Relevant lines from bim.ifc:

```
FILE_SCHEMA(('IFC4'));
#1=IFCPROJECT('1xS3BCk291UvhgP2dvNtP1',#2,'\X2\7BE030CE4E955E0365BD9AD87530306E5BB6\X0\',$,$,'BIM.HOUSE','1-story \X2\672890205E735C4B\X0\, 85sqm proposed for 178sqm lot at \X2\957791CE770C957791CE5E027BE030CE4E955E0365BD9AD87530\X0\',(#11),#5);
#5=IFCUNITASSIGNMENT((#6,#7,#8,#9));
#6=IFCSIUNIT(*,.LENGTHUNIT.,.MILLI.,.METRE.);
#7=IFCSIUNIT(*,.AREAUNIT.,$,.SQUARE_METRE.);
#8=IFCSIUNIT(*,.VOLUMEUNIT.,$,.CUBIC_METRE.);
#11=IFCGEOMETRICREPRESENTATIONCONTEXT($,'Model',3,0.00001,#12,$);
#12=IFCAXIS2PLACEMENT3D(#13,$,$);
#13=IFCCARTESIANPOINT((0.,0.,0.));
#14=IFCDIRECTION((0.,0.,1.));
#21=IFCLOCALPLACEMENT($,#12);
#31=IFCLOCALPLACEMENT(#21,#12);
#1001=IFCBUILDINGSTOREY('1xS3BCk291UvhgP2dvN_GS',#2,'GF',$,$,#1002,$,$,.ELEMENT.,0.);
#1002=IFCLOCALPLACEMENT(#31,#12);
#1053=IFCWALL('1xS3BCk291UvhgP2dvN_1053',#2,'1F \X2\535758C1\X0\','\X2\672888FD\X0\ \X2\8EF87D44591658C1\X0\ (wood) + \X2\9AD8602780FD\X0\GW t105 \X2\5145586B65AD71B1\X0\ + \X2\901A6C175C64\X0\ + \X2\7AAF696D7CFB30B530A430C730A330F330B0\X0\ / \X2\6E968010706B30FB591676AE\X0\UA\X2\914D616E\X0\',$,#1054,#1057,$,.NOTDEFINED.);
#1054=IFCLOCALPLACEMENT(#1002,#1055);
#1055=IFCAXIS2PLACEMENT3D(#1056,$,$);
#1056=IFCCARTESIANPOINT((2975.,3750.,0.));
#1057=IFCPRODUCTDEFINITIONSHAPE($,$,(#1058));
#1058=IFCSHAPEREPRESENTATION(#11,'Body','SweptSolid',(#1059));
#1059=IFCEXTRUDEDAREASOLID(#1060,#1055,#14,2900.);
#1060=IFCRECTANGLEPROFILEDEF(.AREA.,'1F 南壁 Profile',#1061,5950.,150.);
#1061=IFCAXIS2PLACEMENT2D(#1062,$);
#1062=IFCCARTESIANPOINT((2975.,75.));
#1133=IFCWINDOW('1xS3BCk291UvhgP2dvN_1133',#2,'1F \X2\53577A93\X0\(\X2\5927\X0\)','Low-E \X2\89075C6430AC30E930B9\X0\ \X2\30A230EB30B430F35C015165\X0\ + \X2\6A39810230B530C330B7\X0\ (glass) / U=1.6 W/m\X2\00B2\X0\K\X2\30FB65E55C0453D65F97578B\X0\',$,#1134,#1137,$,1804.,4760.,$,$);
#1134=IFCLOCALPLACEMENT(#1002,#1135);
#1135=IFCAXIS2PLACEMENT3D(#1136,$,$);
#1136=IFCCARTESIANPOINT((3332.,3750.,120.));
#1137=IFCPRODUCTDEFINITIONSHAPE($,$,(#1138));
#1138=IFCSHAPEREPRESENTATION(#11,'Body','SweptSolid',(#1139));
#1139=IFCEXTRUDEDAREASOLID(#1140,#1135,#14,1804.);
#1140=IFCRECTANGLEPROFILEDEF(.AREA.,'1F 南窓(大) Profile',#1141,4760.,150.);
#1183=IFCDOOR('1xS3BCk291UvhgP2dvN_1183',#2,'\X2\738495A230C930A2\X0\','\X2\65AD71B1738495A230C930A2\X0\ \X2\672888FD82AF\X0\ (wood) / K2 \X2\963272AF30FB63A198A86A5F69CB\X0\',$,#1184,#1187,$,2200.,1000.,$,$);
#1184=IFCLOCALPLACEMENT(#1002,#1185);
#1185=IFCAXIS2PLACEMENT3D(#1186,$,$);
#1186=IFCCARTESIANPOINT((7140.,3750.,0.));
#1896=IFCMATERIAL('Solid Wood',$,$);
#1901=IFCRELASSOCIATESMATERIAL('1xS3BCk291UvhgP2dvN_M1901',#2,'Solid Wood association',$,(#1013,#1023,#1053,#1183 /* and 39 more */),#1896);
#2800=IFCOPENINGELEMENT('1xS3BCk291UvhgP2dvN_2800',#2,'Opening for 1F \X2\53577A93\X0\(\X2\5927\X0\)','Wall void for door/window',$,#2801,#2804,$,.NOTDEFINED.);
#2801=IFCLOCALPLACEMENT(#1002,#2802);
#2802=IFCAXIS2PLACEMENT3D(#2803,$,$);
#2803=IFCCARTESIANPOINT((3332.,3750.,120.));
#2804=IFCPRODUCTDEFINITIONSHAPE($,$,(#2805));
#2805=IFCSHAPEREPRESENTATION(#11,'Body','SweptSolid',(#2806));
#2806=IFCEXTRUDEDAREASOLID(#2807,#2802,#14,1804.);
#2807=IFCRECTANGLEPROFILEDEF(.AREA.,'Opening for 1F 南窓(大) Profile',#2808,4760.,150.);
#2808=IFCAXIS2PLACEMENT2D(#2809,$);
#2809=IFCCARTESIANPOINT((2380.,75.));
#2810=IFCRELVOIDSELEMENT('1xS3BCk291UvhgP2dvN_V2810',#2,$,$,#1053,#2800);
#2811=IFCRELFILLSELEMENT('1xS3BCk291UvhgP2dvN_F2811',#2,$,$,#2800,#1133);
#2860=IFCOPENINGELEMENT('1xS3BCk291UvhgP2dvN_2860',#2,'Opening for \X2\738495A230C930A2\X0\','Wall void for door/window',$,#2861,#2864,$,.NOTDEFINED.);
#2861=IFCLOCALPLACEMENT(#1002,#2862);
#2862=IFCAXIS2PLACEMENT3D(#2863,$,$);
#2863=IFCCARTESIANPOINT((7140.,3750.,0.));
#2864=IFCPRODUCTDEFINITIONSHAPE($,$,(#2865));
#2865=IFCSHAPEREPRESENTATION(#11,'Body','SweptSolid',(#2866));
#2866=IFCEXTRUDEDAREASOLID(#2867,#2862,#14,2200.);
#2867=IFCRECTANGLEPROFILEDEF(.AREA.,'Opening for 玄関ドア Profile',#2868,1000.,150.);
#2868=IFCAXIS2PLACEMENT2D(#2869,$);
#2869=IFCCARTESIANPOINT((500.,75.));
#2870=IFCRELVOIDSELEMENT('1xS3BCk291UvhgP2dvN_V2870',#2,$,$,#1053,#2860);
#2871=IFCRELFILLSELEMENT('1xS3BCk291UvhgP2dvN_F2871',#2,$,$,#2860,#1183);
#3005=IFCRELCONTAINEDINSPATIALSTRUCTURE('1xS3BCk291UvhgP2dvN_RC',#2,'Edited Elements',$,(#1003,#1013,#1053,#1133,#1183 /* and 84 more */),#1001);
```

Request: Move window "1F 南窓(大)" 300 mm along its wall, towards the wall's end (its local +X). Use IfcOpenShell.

```python
import ifcopenshell
import ifcopenshell.api.geometry
import ifcopenshell.util.placement

model = ifcopenshell.open("bim.ifc")

window = model.by_guid("1xS3BCk291UvhgP2dvN_1133")
opening = window.FillsVoids[0].RelatingOpeningElement
wall = opening.VoidsElements[0].RelatingBuildingElement

wall_matrix = ifcopenshell.util.placement.get_local_placement(wall.ObjectPlacement)
shift = wall_matrix[:3, 0] * 300.0
before = ifcopenshell.util.placement.get_local_placement(window.ObjectPlacement)[:3, 3].copy()

# The window is not placed relative to its opening, so move both.
for product in (opening, window):
    matrix = ifcopenshell.util.placement.get_local_placement(product.ObjectPlacement)
    matrix[:3, 3] += shift
    ifcopenshell.api.geometry.edit_object_placement(model, product=product, matrix=matrix, is_si=False)

after = ifcopenshell.util.placement.get_local_placement(window.ObjectPlacement)[:3, 3]
print("window moved by", (after - before).round(3) + 0.0)

model.write("bim_updated.ifc")
```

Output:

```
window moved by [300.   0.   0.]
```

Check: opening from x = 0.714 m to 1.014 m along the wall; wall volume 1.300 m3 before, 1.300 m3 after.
